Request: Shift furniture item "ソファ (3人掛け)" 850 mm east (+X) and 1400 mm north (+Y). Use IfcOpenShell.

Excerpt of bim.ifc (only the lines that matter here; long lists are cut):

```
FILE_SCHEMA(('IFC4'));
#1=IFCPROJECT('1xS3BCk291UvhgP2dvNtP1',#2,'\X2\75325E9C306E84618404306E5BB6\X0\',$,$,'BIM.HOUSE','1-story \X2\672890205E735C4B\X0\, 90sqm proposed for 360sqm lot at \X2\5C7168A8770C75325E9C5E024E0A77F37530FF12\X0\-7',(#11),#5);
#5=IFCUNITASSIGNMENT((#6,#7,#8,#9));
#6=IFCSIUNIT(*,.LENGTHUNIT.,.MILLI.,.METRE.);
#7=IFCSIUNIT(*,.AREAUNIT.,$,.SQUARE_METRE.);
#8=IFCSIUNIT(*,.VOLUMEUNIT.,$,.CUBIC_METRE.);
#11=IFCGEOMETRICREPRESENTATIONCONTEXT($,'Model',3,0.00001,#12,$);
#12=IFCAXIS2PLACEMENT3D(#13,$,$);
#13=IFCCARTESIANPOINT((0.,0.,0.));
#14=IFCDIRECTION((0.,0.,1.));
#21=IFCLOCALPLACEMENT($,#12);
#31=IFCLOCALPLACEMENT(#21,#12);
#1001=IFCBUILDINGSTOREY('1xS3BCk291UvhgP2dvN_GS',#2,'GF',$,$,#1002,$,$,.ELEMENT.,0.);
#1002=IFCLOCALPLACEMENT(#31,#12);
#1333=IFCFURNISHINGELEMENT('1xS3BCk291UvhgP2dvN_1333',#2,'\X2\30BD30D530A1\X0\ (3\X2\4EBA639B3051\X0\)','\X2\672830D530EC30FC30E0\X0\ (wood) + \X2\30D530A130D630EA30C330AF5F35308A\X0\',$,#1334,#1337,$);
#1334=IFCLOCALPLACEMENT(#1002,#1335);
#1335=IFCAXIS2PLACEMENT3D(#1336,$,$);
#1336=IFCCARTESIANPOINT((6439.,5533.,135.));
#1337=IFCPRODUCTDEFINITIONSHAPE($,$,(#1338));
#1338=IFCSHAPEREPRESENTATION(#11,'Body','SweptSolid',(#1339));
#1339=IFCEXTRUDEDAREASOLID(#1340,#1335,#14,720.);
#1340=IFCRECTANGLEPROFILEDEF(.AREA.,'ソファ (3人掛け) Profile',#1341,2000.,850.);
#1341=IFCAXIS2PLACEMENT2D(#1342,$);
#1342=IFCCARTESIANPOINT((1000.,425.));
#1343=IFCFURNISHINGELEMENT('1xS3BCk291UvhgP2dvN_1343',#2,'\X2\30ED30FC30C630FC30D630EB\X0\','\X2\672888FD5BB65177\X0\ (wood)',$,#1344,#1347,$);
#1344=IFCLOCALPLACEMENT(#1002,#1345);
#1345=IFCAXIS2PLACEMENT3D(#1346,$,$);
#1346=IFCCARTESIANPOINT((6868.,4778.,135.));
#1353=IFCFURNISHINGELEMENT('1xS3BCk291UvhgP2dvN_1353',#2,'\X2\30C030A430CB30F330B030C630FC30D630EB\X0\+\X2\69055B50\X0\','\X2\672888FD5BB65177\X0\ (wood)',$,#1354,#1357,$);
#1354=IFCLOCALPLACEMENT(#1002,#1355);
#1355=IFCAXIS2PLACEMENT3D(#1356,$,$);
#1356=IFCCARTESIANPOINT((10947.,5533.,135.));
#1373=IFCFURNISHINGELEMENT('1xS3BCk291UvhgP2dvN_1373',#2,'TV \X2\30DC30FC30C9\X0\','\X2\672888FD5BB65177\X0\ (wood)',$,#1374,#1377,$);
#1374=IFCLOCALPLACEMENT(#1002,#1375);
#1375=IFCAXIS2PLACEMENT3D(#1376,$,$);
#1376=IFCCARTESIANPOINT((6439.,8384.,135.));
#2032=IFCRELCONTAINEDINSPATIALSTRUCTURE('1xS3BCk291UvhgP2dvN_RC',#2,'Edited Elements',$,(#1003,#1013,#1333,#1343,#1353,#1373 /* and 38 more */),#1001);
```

```python
import ifcopenshell
import ifcopenshell.api.geometry
import ifcopenshell.util.placement
import ifcopenshell.util.unit

model = ifcopenshell.open("bim.ifc")
unit_scale = ifcopenshell.util.unit.calculate_unit_scale(model)

item = model.by_guid("1xS3BCk291UvhgP2dvN_1333")
matrix = ifcopenshell.util.placement.get_local_placement(item.ObjectPlacement)
matrix[0, 3] += 0.85 / unit_scale
matrix[1, 3] += 1.4 / unit_scale
ifcopenshell.api.geometry.edit_object_placement(model, product=item, matrix=matrix, is_si=False)

print(ifcopenshell.util.placement.get_local_placement(item.ObjectPlacement).round(3) + 0.0)

model.write("bim_edited.ifc")
```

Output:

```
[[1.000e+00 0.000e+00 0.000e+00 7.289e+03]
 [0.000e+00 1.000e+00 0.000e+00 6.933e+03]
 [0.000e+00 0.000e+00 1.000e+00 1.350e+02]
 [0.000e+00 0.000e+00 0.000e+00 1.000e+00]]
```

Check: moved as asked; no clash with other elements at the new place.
